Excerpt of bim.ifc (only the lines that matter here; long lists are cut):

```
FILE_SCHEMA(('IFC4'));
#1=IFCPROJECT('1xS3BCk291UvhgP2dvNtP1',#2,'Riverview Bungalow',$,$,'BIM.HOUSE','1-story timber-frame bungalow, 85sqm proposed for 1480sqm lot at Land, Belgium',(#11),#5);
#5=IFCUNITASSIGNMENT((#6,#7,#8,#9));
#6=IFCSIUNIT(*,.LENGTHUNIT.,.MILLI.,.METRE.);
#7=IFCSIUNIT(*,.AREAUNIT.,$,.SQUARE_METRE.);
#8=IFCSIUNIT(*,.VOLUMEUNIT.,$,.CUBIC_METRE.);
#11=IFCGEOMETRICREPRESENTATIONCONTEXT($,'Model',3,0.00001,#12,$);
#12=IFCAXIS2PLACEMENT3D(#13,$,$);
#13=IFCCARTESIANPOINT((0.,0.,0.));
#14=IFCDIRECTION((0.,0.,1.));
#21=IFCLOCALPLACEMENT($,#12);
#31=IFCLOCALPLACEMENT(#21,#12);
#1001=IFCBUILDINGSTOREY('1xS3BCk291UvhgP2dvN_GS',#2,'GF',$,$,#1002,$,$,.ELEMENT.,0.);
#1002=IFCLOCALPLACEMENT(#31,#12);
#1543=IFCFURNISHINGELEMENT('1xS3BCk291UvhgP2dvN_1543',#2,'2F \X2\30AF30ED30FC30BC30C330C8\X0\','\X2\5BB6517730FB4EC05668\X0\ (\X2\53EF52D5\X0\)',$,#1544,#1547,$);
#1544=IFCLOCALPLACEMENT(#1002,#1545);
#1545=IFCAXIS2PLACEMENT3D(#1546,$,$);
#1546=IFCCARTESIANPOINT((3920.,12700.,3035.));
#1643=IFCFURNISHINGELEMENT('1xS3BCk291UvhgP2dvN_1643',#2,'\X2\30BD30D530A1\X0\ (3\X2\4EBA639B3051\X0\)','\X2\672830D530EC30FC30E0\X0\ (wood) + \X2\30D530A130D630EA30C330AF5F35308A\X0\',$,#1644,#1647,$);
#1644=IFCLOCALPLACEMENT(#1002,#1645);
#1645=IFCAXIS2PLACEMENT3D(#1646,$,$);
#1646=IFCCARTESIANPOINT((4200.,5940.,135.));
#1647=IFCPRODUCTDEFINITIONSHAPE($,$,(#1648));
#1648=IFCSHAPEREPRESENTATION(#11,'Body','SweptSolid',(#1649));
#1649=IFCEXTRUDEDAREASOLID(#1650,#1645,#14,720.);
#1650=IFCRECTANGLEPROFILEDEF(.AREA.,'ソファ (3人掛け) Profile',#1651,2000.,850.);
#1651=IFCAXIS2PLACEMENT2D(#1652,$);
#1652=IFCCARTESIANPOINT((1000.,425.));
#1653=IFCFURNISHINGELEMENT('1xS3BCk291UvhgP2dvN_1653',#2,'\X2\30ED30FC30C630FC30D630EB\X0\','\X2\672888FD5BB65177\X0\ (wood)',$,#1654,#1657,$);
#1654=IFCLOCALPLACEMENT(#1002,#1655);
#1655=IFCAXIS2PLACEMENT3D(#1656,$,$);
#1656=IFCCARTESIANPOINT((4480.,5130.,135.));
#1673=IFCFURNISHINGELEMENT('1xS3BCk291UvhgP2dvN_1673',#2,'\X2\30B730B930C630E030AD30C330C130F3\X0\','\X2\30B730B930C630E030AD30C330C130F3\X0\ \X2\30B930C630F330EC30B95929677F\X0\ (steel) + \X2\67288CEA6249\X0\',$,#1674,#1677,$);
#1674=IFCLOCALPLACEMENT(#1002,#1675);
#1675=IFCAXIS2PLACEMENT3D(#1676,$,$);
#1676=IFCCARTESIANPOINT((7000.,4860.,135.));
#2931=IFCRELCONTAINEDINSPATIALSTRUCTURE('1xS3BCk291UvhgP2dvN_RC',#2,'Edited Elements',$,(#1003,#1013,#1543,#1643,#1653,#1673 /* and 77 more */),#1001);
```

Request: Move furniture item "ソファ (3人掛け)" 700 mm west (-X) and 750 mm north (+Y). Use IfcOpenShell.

```python
import ifcopenshell
import ifcopenshell.api.geometry
import ifcopenshell.util.placement

model = ifcopenshell.open("bim.ifc")

item = model.by_id(1643)
matrix = ifcopenshell.util.placement.get_local_placement(item.ObjectPlacement)
matrix[0, 3] -= 700.0
matrix[1, 3] += 750.0
ifcopenshell.api.geometry.edit_object_placement(model, product=item, matrix=matrix, is_si=False)

print(ifcopenshell.util.placement.get_local_placement(item.ObjectPlacement).round(3) + 0.0)

model.write("bim_v2.ifc")
```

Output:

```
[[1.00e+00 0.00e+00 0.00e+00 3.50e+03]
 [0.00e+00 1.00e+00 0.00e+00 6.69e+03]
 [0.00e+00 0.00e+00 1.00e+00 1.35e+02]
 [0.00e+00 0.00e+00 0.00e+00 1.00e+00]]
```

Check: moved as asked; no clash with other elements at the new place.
